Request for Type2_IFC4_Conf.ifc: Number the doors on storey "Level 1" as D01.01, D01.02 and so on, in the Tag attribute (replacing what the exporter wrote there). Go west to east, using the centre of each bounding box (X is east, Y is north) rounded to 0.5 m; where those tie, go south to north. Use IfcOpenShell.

First a look at what the model holds.

```python
import ifcopenshell
import ifcopenshell.util.element
import ifcopenshell.util.placement

model = ifcopenshell.open("Type2_IFC4_Conf.ifc")
print(model.schema)
storey = next(s for s in model.by_type("IfcBuildingStorey") if s.Name == "Level 1")
doors = [e for e in ifcopenshell.util.element.get_decomposition(storey) if e.is_a("IfcDoor")]
for e in sorted(doors, key=lambda e: e.id()):
    origin = ifcopenshell.util.placement.get_local_placement(e.ObjectPlacement)[:3, 3]
    print(e.id(), e.Tag, e.Name, origin.round(2) + 0.0, sep=" | ")
```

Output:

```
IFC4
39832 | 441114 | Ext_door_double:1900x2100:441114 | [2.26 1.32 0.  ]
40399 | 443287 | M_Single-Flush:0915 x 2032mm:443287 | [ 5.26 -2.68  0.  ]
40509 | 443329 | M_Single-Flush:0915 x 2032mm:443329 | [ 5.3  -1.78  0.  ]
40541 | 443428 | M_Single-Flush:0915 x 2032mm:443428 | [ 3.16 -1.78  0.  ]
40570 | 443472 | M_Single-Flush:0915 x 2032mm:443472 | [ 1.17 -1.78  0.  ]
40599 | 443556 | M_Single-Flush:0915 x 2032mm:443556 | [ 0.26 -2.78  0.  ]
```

```python
import ifcopenshell
import ifcopenshell.geom
import ifcopenshell.util.element
import ifcopenshell.util.shape

model = ifcopenshell.open("Type2_IFC4_Conf.ifc")
settings = ifcopenshell.geom.settings()
settings.set("use-world-coords", True)


def centre(element):
    shape = ifcopenshell.geom.create_shape(settings, element)
    return ifcopenshell.util.shape.get_bbox_centroid(shape.geometry)


storey = next(s for s in model.by_type("IfcBuildingStorey") if s.Name == "Level 1")
doors = [e for e in ifcopenshell.util.element.get_decomposition(storey) if e.is_a("IfcDoor")]

# Insertion points can sit at a corner or the storey origin, so sort by the geometry (in metres).
centres = {e: centre(e) for e in doors}
doors.sort(key=lambda e: (round(centres[e][0] / 0.5), centres[e][1]))

for i, e in enumerate(doors, start=1):
    number = f"D01.{i:02d}"
    e.Tag = number
    print(e.id(), number)

model.write("Type2_IFC4_Conf_rev.ifc")
```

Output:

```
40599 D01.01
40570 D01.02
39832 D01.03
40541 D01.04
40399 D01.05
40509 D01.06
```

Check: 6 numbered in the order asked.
